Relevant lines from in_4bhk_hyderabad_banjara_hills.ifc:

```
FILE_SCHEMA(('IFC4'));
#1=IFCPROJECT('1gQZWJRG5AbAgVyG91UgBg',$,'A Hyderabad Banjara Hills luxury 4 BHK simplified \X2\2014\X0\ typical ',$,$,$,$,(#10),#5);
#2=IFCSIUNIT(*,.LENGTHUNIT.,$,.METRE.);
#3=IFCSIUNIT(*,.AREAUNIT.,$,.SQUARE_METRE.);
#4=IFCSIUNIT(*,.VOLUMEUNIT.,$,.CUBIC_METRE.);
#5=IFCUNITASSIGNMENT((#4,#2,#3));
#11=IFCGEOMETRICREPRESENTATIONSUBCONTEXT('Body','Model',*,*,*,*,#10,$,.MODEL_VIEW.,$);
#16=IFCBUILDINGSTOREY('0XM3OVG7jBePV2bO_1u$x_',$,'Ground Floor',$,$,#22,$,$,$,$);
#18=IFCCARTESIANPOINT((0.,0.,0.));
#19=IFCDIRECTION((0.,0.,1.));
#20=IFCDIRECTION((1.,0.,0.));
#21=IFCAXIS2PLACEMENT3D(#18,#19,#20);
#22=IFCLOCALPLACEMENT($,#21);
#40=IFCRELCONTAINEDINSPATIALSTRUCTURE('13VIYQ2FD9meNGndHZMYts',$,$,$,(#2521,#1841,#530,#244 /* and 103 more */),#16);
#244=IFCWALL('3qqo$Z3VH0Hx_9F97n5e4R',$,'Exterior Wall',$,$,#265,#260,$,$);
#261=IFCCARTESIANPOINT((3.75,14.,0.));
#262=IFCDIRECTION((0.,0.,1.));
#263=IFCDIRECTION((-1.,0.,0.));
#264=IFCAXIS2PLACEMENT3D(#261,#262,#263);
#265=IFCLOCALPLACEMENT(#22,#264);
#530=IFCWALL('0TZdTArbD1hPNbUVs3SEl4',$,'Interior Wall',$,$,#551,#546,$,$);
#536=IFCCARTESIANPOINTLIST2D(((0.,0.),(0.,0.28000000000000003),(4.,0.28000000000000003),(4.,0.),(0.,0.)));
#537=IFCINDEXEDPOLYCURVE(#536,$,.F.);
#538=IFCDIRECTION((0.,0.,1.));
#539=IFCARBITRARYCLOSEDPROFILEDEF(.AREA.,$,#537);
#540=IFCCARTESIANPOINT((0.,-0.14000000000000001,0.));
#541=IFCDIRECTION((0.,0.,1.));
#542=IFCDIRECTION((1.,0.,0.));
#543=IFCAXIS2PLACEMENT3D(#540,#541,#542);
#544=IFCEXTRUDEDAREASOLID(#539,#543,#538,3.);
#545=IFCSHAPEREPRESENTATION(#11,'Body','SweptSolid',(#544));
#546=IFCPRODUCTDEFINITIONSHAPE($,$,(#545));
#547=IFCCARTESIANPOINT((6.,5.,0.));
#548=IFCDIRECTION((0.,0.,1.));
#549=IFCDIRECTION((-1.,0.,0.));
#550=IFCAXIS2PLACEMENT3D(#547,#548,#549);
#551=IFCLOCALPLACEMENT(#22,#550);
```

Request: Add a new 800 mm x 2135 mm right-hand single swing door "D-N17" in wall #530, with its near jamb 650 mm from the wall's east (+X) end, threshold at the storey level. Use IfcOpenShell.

```python
import numpy as np
import ifcopenshell
import ifcopenshell.api.feature
import ifcopenshell.api.geometry
import ifcopenshell.api.root
import ifcopenshell.api.spatial
import ifcopenshell.geom
import ifcopenshell.util.element
import ifcopenshell.util.placement
import ifcopenshell.util.representation
import ifcopenshell.util.shape
import ifcopenshell.util.unit

model = ifcopenshell.open("in_4bhk_hyderabad_banjara_hills.ifc")
unit_scale = ifcopenshell.util.unit.calculate_unit_scale(model)
settings = ifcopenshell.geom.settings()


def volume(element):
    """Net volume in cubic metres, openings subtracted."""
    shape = ifcopenshell.geom.create_shape(settings, element)
    return ifcopenshell.util.shape.get_volume(shape.geometry)


wall = model.by_id(530)
storey = ifcopenshell.util.element.get_container(wall, ifc_class="IfcBuildingStorey")
context = ifcopenshell.util.representation.get_context(model, "Model", "Body", "MODEL_VIEW")
before = volume(wall)

width, height, from_end, sill = 0.8, 2.135, 0.65, 0.0  # metres

# The wall runs along its own X axis, and the end named is its -X end.
wall_shape = ifcopenshell.geom.create_shape(settings, wall)
x, y, z = ifcopenshell.util.shape.get_vertices(wall_shape.geometry).T
start = x.min() + from_end
face, thickness = float(y.min()), float(y.max() - y.min())
wall_matrix = ifcopenshell.util.placement.get_local_placement(wall.ObjectPlacement)
level = ifcopenshell.util.placement.get_local_placement(storey.ObjectPlacement)[2, 3]


def in_wall(x, y):
    """Placement at x, y metres in the wall's axes, at sill height."""
    matrix = wall_matrix.copy()
    matrix[:, 3] = wall_matrix @ np.array([x / unit_scale, y / unit_scale, 0.0, 1.0])
    matrix[2, 3] = level + sill / unit_scale
    return matrix


# Opening: a box that overshoots both wall faces by 50 mm.
opening = ifcopenshell.api.root.create_entity(model, ifc_class="IfcOpeningElement", predefined_type="OPENING")
box = ifcopenshell.api.geometry.add_wall_representation(
    model, context=context, length=width, height=height, thickness=thickness + 0.1
)
ifcopenshell.api.geometry.assign_representation(model, product=opening, representation=box)
ifcopenshell.api.geometry.edit_object_placement(model, product=opening, matrix=in_wall(start, face - 0.05), is_si=False)
ifcopenshell.api.feature.add_feature(model, feature=opening, element=wall)

door = ifcopenshell.api.root.create_entity(model, ifc_class="IfcDoor", name="D-N17", predefined_type="DOOR")
door.OverallWidth, door.OverallHeight = width / unit_scale, height / unit_scale
door.OperationType = "SINGLE_SWING_RIGHT"
body = ifcopenshell.api.geometry.add_door_representation(
    model,
    context=context,
    overall_width=door.OverallWidth,
    overall_height=door.OverallHeight,
    operation_type="SINGLE_SWING_RIGHT",
    lining_properties={"LiningDepth": thickness / unit_scale, "ThresholdDepth": thickness / unit_scale},
)
ifcopenshell.api.geometry.assign_representation(model, product=door, representation=body)
ifcopenshell.api.spatial.assign_container(model, products=[door], relating_structure=storey)
ifcopenshell.api.feature.add_filling(model, opening=opening, element=door)

# The lining spans the wall, so the door starts at the wall face.
ifcopenshell.api.geometry.edit_object_placement(model, product=door, matrix=in_wall(start, face), is_si=False)

after = volume(wall)

print(f"wall volume {before:.3f} -> {after:.3f} m3")

model.write("in_4bhk_hyderabad_banjara_hills_v2.ifc")
```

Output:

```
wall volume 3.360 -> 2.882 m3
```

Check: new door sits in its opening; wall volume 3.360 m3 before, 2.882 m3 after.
